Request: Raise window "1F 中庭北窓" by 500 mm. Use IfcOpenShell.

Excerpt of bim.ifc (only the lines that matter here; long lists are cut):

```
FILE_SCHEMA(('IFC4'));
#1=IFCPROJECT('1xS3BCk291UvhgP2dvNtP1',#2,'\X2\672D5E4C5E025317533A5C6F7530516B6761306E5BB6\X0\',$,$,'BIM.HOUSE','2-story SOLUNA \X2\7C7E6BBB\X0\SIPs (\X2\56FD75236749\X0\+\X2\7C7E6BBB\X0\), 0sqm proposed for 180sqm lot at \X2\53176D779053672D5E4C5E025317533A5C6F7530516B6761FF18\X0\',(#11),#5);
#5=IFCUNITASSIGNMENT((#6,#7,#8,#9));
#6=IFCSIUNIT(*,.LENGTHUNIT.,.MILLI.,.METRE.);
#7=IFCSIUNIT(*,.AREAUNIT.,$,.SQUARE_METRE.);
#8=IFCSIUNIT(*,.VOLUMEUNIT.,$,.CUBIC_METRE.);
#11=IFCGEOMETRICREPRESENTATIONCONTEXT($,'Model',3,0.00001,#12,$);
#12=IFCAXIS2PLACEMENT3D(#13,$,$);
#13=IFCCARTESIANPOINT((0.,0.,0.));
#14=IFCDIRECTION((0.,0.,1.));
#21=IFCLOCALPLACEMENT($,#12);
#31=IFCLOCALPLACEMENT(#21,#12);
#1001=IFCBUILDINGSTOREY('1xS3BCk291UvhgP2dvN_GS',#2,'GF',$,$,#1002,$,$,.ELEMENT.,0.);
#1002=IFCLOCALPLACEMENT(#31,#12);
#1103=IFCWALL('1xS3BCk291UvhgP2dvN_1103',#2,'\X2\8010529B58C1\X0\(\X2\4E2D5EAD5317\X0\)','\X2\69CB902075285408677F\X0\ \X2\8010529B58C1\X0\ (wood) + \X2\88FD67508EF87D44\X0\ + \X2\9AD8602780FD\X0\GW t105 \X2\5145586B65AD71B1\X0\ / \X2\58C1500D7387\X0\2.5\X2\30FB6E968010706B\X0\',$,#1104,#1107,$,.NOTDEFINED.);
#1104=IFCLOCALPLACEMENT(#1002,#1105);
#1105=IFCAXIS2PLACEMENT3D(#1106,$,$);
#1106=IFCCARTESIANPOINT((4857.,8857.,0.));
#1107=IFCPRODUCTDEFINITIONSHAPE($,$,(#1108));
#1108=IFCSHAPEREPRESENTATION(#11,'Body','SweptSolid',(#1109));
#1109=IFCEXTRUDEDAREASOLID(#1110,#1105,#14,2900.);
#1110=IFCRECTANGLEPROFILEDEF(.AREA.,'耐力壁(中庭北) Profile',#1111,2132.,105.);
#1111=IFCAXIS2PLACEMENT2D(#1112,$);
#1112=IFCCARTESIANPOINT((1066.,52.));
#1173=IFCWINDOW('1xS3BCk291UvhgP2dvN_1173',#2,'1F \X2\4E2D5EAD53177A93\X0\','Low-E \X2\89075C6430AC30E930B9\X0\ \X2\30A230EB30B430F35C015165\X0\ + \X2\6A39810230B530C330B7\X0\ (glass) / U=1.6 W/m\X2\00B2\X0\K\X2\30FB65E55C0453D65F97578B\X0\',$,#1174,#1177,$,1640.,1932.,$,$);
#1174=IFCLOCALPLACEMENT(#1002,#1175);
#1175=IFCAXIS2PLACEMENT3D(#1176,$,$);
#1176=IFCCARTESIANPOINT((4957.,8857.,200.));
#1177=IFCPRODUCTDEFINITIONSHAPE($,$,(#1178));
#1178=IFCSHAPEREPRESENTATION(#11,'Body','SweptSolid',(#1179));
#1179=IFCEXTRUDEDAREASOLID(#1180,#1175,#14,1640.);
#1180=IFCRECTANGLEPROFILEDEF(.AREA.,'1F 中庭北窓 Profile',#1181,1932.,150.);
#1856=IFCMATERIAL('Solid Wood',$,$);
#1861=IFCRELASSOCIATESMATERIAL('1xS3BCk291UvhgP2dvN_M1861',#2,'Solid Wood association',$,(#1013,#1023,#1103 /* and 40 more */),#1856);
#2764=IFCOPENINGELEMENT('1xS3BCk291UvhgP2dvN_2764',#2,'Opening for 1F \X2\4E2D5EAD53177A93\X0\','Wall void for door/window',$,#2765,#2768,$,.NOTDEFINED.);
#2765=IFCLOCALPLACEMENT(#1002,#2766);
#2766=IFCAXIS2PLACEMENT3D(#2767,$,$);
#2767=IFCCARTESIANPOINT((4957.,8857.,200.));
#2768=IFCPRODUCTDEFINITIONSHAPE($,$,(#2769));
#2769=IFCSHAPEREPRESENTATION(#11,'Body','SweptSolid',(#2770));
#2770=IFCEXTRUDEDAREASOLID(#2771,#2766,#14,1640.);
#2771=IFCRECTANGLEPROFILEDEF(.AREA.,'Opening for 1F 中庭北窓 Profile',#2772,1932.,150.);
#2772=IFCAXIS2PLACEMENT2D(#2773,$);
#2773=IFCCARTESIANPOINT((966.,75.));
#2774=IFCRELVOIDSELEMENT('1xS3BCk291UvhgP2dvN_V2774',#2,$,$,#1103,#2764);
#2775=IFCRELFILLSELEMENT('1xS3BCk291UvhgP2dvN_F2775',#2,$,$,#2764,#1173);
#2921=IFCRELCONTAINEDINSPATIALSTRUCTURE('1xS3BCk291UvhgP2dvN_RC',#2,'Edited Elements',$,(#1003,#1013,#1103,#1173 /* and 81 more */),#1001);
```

```python
import numpy as np
import ifcopenshell
import ifcopenshell.api.geometry
import ifcopenshell.util.placement
import ifcopenshell.util.unit

model = ifcopenshell.open("bim.ifc")
unit_scale = ifcopenshell.util.unit.calculate_unit_scale(model)

window = model.by_id(1173)
opening = window.FillsVoids[0].RelatingOpeningElement
dz = 0.5 / unit_scale

shift = np.array([0.0, 0.0, dz])
# The window is not placed relative to its opening, so move both.
for product in (opening, window):
    matrix = ifcopenshell.util.placement.get_local_placement(product.ObjectPlacement)
    matrix[:3, 3] += shift
    ifcopenshell.api.geometry.edit_object_placement(model, product=product, matrix=matrix, is_si=False)

print(f"moved by {dz * unit_scale:+.3f} m")

model.write("bim_rev.ifc")
```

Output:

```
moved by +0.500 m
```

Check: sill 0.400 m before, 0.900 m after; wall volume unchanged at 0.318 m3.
